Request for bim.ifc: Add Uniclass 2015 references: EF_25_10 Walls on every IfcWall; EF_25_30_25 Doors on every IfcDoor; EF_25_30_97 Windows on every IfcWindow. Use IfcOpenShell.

First a look at what the model holds.

```python
import ifcopenshell

model = ifcopenshell.open("bim.ifc")
print(model.schema)
print("classifications:", [c.Name for c in model.by_type("IfcClassification")])
for ifc_class in ("IfcDoor", "IfcRoof", "IfcStair", "IfcWall", "IfcWindow"):
    print(ifc_class, len(model.by_type(ifc_class)))
```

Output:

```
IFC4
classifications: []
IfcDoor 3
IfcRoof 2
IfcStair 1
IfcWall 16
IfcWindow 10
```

```python
import ifcopenshell
import ifcopenshell.api.classification

model = ifcopenshell.open("bim.ifc")

system = ifcopenshell.api.classification.add_classification(model, classification="Uniclass 2015")

codes = {
    "IfcWall": ("EF_25_10", "Walls"),
    "IfcDoor": ("EF_25_30_25", "Doors"),
    "IfcWindow": ("EF_25_30_97", "Windows"),
}
for ifc_class, (code, name) in codes.items():
    products = model.by_type(ifc_class)
    ifcopenshell.api.classification.add_reference(
        model, products=products, classification=system, identification=code, name=name
    )
    print(code, len(products))

model.write("bim_updated.ifc")
```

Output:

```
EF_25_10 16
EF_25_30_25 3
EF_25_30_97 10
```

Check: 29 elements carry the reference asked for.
